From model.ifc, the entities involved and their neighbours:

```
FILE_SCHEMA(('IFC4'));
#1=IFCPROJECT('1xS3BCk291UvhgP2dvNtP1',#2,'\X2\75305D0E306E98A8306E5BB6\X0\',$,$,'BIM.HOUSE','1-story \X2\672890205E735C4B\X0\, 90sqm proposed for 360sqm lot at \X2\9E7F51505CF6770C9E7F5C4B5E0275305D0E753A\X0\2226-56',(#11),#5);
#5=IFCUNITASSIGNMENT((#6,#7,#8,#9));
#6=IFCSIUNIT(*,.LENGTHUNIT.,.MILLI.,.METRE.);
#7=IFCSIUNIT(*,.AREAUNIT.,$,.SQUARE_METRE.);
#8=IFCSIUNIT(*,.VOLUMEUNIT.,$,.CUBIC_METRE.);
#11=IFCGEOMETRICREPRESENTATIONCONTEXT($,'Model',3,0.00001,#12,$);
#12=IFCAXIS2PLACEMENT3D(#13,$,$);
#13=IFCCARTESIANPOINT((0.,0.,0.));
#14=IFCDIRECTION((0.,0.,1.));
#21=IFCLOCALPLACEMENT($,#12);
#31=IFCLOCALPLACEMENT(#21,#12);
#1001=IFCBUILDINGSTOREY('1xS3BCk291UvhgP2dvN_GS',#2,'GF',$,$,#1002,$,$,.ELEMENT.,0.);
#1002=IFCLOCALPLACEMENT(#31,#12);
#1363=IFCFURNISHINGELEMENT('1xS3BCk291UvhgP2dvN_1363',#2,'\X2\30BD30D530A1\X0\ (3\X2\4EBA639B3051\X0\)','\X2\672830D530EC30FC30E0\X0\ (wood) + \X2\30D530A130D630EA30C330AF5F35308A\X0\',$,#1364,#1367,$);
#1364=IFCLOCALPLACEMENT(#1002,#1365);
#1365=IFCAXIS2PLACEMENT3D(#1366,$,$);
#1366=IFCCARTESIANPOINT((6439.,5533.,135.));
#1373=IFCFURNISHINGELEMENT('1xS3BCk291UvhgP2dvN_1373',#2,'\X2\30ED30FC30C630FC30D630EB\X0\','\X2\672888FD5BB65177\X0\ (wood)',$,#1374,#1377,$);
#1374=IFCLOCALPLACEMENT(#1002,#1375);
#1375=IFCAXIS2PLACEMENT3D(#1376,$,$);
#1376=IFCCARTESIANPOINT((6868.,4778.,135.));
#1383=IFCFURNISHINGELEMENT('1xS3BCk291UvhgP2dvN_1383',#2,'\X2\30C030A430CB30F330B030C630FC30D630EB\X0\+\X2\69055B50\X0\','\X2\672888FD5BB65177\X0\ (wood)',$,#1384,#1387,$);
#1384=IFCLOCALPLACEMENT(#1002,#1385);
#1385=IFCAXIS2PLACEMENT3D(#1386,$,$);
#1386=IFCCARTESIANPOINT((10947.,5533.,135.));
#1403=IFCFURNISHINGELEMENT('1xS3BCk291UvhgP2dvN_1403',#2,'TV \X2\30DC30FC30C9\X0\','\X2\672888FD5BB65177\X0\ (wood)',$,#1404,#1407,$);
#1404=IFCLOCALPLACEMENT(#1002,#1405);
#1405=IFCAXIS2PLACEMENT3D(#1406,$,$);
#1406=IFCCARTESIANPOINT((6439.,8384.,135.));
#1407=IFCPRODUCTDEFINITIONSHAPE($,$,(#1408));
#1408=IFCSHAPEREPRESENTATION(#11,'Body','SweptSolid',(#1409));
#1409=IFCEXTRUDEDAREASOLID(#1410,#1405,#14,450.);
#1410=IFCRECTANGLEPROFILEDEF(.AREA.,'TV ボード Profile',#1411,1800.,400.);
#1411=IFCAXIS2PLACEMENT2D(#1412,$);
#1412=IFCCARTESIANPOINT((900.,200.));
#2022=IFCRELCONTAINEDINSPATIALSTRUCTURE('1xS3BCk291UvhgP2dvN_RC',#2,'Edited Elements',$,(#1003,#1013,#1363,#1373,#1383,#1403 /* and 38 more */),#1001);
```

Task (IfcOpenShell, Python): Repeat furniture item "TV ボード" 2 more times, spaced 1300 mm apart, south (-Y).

```python
import numpy as np
import ifcopenshell
import ifcopenshell.api.geometry
import ifcopenshell.api.root
import ifcopenshell.util.element
import ifcopenshell.util.placement

model = ifcopenshell.open("model.ifc")


def reuse_history(source, copy):
    """copy_class also copies each property set's owner history, people and application; keep the originals."""
    for rel in copy.IsDefinedBy:
        if rel.is_a("IfcRelDefinesByProperties") and (history := rel.RelatingPropertyDefinition.OwnerHistory):
            rel.RelatingPropertyDefinition.OwnerHistory = source.OwnerHistory
            ifcopenshell.util.element.remove_deep2(model, history)


source = model.by_id(1403)
base = ifcopenshell.util.placement.get_local_placement(source.ObjectPlacement)
step = np.array([0.0, -1.0, 0.0]) * 1300.0

for i in range(1, 3):
    copy = ifcopenshell.api.root.copy_class(model, product=source)
    copy.Representation = ifcopenshell.util.element.copy_deep(
        model, source.Representation, exclude=["IfcGeometricRepresentationContext", "IfcRepresentationMap"]
    )
    reuse_history(source, copy)
    matrix = base.copy()
    matrix[:3, 3] += i * step
    print("added at", matrix[:3, 3].round(3) + 0.0)
    ifcopenshell.api.geometry.edit_object_placement(model, product=copy, matrix=matrix, is_si=False)

model.write("model_updated.ifc")
```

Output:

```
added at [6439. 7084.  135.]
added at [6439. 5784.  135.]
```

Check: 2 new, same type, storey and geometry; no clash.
